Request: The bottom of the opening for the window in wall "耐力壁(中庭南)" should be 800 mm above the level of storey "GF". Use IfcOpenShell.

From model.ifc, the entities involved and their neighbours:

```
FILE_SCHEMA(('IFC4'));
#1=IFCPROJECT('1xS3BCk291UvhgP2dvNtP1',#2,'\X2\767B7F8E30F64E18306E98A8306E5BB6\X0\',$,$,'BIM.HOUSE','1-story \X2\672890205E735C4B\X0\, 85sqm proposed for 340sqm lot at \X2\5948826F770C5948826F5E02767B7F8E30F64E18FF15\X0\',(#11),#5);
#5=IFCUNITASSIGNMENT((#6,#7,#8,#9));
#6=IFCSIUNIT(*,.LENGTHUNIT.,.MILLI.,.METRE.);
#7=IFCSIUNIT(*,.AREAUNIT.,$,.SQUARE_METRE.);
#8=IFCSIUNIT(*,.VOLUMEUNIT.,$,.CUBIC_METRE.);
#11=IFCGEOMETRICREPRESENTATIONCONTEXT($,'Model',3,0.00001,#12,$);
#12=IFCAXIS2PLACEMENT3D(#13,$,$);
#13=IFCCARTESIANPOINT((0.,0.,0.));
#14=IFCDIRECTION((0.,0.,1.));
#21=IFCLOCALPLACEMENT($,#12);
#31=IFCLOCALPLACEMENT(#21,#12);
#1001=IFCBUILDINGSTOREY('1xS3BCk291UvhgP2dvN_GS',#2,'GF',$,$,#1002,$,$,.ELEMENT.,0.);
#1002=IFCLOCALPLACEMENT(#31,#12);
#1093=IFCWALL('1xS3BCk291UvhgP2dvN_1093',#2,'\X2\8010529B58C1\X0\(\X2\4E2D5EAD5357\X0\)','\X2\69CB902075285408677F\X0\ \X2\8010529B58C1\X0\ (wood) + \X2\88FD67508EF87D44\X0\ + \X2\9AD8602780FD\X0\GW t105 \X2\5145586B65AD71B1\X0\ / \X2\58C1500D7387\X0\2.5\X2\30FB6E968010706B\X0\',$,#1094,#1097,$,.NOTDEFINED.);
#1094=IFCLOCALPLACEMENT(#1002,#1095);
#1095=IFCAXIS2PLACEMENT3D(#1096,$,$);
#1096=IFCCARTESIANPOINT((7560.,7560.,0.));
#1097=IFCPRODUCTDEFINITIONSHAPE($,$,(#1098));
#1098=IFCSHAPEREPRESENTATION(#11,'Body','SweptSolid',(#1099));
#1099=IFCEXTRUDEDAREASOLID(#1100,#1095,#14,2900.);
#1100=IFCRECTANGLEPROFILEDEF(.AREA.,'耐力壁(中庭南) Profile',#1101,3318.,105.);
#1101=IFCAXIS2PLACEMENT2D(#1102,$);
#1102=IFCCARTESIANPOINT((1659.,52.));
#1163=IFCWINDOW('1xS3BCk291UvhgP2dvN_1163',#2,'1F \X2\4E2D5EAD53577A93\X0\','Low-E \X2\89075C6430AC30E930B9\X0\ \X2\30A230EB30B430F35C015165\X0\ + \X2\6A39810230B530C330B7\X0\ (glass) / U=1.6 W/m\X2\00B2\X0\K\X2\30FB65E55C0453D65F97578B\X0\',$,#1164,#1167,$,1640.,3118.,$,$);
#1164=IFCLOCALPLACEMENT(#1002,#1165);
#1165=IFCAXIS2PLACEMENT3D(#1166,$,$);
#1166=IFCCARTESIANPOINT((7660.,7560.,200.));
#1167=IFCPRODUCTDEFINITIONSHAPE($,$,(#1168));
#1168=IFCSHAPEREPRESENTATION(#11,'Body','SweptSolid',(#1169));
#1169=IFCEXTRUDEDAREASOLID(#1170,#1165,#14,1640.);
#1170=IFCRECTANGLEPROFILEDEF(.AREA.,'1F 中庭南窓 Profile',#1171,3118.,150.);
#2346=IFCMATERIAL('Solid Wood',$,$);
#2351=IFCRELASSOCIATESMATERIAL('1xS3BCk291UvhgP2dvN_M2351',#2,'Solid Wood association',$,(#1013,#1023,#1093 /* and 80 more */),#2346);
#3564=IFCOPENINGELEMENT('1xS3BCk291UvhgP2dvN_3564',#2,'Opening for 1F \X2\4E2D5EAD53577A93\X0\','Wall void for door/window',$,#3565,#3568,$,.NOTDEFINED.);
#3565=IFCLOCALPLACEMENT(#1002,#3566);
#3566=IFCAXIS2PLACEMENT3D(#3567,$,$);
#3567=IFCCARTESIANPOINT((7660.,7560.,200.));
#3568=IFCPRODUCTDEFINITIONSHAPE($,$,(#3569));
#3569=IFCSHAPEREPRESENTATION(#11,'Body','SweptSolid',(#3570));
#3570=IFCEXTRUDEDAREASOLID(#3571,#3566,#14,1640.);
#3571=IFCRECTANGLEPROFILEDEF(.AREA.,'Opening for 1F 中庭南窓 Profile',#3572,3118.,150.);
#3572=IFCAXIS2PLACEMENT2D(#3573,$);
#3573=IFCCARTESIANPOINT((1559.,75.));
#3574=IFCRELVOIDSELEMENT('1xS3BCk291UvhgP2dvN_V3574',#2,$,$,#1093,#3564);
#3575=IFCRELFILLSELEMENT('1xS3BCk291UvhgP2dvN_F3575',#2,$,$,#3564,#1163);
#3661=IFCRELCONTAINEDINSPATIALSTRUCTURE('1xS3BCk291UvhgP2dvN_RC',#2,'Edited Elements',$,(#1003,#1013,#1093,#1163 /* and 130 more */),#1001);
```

```python
import numpy as np
import ifcopenshell
import ifcopenshell.api.geometry
import ifcopenshell.geom
import ifcopenshell.util.element
import ifcopenshell.util.placement
import ifcopenshell.util.shape
import ifcopenshell.util.unit

model = ifcopenshell.open("model.ifc")
unit_scale = ifcopenshell.util.unit.calculate_unit_scale(model)

window = model.by_guid("1xS3BCk291UvhgP2dvN_1163")
opening = window.FillsVoids[0].RelatingOpeningElement
storey = ifcopenshell.util.element.get_container(window, ifc_class="IfcBuildingStorey")
level = ifcopenshell.util.placement.get_local_placement(storey.ObjectPlacement)[2, 3]

# The opening's origin need not be at the sill, so measure its lowest point.
shape = ifcopenshell.geom.create_shape(ifcopenshell.geom.settings(), opening)
bottom = ifcopenshell.util.shape.get_shape_bottom_elevation(shape, shape.geometry) / unit_scale
dz = level + 0.8 / unit_scale - bottom

shift = np.array([0.0, 0.0, dz])
# The window is not placed relative to its opening, so move both.
for product in (opening, window):
    matrix = ifcopenshell.util.placement.get_local_placement(product.ObjectPlacement)
    matrix[:3, 3] += shift
    ifcopenshell.api.geometry.edit_object_placement(model, product=product, matrix=matrix, is_si=False)

print(f"moved by {dz * unit_scale:+.3f} m")

model.write("model_edited.ifc")
```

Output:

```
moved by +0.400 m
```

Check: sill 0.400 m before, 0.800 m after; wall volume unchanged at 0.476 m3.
